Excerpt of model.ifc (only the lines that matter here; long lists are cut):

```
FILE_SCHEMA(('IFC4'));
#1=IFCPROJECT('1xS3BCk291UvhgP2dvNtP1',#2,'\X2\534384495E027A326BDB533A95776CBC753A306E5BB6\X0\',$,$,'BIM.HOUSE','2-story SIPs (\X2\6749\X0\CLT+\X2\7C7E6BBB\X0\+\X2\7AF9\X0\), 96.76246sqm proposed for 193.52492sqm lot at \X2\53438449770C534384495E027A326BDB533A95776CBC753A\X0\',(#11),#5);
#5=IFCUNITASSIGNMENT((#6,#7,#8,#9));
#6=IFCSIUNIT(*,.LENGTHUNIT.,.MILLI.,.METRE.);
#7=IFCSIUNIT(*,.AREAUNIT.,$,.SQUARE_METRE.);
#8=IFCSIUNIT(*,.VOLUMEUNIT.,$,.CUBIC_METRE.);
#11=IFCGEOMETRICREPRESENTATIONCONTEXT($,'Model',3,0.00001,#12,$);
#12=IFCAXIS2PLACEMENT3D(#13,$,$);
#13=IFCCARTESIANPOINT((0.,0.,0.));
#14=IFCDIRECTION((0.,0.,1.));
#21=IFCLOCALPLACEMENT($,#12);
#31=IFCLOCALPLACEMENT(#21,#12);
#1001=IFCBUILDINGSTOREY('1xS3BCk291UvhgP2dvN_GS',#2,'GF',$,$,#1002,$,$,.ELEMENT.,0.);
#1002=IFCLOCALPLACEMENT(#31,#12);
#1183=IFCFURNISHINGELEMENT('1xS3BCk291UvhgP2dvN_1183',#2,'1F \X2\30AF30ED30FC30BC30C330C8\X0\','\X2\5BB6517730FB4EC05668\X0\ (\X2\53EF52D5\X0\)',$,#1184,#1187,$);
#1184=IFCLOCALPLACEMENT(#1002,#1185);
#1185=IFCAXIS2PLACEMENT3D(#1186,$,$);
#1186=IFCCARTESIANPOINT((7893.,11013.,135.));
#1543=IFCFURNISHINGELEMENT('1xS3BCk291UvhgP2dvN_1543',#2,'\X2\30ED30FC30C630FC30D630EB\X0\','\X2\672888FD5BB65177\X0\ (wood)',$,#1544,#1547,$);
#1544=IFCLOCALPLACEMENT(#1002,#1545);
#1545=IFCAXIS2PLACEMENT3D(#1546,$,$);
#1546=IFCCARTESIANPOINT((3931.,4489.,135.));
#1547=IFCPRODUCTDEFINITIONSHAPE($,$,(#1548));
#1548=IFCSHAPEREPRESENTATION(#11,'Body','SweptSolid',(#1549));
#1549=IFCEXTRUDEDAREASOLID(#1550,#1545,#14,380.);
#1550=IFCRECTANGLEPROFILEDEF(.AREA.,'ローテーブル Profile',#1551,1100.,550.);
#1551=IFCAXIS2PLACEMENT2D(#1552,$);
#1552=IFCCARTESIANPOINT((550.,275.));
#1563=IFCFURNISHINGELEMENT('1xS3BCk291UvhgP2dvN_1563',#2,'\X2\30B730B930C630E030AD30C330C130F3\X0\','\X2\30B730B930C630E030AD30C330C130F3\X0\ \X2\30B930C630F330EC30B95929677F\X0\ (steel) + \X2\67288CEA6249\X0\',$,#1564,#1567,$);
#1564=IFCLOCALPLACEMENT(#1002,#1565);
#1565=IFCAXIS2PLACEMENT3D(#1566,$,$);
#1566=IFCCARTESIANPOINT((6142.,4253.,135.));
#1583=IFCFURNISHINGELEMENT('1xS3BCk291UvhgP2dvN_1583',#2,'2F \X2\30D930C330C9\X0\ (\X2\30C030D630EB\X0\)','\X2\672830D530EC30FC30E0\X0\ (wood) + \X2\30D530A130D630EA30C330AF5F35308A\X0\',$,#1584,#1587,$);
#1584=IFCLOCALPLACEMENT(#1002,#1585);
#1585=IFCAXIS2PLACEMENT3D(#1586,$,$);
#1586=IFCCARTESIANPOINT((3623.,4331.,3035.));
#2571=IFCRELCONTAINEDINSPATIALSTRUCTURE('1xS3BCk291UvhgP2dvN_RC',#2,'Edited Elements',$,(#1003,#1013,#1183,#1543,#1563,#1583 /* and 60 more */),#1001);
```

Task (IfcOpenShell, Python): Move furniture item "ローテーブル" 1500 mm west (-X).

```python
import ifcopenshell
import ifcopenshell.api.geometry
import ifcopenshell.util.placement
import ifcopenshell.util.unit

model = ifcopenshell.open("model.ifc")
unit_scale = ifcopenshell.util.unit.calculate_unit_scale(model)

item = model.by_id(1543)
matrix = ifcopenshell.util.placement.get_local_placement(item.ObjectPlacement)
matrix[0, 3] -= 1.5 / unit_scale
ifcopenshell.api.geometry.edit_object_placement(model, product=item, matrix=matrix, is_si=False)

print(ifcopenshell.util.placement.get_local_placement(item.ObjectPlacement).round(3) + 0.0)

model.write("model_edited.ifc")
```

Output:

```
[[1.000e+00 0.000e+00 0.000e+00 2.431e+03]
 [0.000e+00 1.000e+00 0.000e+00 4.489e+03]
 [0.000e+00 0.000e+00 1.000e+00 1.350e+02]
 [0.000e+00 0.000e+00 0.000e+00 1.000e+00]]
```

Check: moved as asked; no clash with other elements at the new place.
